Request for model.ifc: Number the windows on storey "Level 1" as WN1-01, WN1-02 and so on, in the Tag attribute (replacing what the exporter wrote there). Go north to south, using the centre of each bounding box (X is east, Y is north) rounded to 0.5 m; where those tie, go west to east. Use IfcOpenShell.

First a look at what the model holds.

```python
import ifcopenshell
import ifcopenshell.util.element
import ifcopenshell.util.placement

model = ifcopenshell.open("model.ifc")
print(model.schema)
storey = next(s for s in model.by_type("IfcBuildingStorey") if s.Name == "Level 1")
windows = [e for e in ifcopenshell.util.element.get_decomposition(storey) if e.is_a("IfcWindow")]
for e in sorted(windows, key=lambda e: e.id()):
    origin = ifcopenshell.util.placement.get_local_placement(e.ObjectPlacement)[:3, 3]
    print(e.id(), e.Tag, e.Name, origin.round(2) + 0.0, sep=" | ")
```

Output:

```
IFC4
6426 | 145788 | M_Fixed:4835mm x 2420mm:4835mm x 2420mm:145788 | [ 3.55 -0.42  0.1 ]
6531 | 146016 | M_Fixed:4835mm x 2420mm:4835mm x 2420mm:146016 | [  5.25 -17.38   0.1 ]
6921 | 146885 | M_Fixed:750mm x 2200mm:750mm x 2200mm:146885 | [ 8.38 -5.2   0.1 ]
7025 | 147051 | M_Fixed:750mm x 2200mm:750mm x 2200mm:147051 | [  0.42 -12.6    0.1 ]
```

```python
import ifcopenshell
import ifcopenshell.geom
import ifcopenshell.util.element
import ifcopenshell.util.shape

model = ifcopenshell.open("model.ifc")
settings = ifcopenshell.geom.settings()
settings.set("use-world-coords", True)


def centre(element):
    shape = ifcopenshell.geom.create_shape(settings, element)
    return ifcopenshell.util.shape.get_bbox_centroid(shape.geometry)


storey = next(s for s in model.by_type("IfcBuildingStorey") if s.Name == "Level 1")
windows = [e for e in ifcopenshell.util.element.get_decomposition(storey) if e.is_a("IfcWindow")]

# Insertion points can sit at a corner or the storey origin, so sort by the geometry (in metres).
centres = {e: centre(e) for e in windows}
windows.sort(key=lambda e: (-round(centres[e][1] / 0.5), centres[e][0]))

for i, e in enumerate(windows, start=1):
    number = f"WN1-{i:02d}"
    e.Tag = number
    print(e.id(), number)

model.write("model_updated.ifc")
```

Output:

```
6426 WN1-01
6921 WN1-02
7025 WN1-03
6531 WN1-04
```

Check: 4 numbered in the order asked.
